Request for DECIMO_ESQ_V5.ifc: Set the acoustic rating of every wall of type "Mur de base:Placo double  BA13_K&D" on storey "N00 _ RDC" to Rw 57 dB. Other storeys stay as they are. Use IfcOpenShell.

First a look at what the model holds.

```python
import ifcopenshell
import ifcopenshell.util.element

model = ifcopenshell.open("DECIMO_ESQ_V5.ifc")
print(model.schema)
storey = next(s for s in model.by_type("IfcBuildingStorey") if s.Name == "N00 _ RDC")
walls = [e for e in ifcopenshell.util.element.get_decomposition(storey) if e.is_a("IfcWall")]
seen = {}
for e in walls:
    element_type = ifcopenshell.util.element.get_type(e)
    key = (element_type.Name if element_type != e and element_type else None, ifcopenshell.util.element.get_pset(e, "Pset_WallCommon", "AcousticRating"))
    seen[key] = seen.get(key, 0) + 1
for (name, value), count in sorted(seen.items(), key=str):
    print(count, "x", name, "|", value)
```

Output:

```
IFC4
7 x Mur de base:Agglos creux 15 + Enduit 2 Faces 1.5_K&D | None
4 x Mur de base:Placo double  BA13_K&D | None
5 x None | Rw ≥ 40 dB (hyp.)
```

```python
import ifcopenshell
import ifcopenshell.api.pset
import ifcopenshell.util.element

model = ifcopenshell.open("DECIMO_ESQ_V5.ifc")

storey = next(s for s in model.by_type("IfcBuildingStorey") if s.Name == "N00 _ RDC")
walls = [e for e in ifcopenshell.util.element.get_decomposition(storey) if e.is_a("IfcWall")]

count = 0
for e in walls:
    element_type = ifcopenshell.util.element.get_type(e)
    if element_type in (None, e) or element_type.Name != "Mur de base:Placo double  BA13_K&D":
        continue
    # add_pset returns the element's existing set when there is one.
    pset = ifcopenshell.api.pset.add_pset(model, product=e, name="Pset_WallCommon")
    ifcopenshell.api.pset.edit_pset(model, pset=pset, properties={"AcousticRating": "Rw 57 dB"})
    count += 1

print(count, "walls updated")

model.write("DECIMO_ESQ_V5_rev.ifc")
```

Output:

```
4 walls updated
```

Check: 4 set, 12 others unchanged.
